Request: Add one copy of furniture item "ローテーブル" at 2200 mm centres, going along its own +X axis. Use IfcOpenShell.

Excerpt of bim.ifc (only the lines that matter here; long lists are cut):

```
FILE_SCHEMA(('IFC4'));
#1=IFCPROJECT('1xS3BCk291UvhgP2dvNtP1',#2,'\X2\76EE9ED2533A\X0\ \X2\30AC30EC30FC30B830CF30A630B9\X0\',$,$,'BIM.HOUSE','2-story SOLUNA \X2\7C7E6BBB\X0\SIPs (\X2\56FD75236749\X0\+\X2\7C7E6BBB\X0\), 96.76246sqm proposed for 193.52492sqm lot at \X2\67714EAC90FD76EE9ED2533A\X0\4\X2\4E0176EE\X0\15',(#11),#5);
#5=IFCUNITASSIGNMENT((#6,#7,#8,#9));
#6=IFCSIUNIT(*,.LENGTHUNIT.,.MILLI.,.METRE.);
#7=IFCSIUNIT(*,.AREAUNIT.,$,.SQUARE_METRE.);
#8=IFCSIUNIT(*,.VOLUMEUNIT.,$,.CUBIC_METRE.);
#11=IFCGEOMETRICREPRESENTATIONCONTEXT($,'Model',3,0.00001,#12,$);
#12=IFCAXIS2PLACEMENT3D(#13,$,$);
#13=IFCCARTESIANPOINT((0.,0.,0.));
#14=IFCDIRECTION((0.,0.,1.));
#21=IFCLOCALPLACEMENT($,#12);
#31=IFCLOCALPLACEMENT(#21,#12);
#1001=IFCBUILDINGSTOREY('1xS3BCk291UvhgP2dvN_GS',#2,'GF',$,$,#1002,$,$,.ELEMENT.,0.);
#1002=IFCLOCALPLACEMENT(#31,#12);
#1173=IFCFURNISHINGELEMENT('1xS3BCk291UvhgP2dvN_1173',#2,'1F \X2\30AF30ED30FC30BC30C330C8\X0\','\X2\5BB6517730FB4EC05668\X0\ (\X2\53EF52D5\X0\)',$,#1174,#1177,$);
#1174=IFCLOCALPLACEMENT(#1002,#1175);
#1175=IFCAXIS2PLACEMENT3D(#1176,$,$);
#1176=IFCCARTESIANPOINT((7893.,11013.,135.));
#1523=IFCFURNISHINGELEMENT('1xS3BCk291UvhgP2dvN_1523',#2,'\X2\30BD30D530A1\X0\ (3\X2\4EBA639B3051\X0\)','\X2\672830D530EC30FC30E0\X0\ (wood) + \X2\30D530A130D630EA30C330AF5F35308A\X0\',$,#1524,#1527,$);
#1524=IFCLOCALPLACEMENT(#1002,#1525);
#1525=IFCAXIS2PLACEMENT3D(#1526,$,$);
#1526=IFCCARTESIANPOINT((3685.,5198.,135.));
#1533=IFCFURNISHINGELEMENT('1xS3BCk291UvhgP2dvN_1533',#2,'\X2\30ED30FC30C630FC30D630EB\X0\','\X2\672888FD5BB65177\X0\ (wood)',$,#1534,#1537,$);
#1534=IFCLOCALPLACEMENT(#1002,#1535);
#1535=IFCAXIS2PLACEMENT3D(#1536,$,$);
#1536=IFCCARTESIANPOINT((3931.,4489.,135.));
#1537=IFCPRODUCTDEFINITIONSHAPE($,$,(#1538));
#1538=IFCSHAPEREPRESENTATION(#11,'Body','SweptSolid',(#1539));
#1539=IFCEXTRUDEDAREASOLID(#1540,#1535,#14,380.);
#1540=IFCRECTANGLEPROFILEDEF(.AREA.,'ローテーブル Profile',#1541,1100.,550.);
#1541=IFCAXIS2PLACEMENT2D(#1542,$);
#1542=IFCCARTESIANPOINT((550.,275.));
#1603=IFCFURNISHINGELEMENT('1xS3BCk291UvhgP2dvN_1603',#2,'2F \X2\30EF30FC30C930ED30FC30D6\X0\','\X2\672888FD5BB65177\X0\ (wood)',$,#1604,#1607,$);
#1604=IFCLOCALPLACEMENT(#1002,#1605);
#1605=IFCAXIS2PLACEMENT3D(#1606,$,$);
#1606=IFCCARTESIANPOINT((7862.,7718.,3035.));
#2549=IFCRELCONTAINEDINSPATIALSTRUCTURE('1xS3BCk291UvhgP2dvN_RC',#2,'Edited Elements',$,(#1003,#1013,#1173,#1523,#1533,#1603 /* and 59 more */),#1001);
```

```python
import ifcopenshell
import ifcopenshell.api.geometry
import ifcopenshell.api.root
import ifcopenshell.util.element
import ifcopenshell.util.placement

model = ifcopenshell.open("bim.ifc")


def reuse_history(source, copy):
    """copy_class also copies each property set's owner history, people and application; keep the originals."""
    for rel in copy.IsDefinedBy:
        if rel.is_a("IfcRelDefinesByProperties") and (history := rel.RelatingPropertyDefinition.OwnerHistory):
            rel.RelatingPropertyDefinition.OwnerHistory = source.OwnerHistory
            ifcopenshell.util.element.remove_deep2(model, history)


source = model.by_guid("1xS3BCk291UvhgP2dvN_1533")
base = ifcopenshell.util.placement.get_local_placement(source.ObjectPlacement)
step = base[:3, 0] * 2200.0

for i in range(1, 2):
    copy = ifcopenshell.api.root.copy_class(model, product=source)
    copy.Representation = ifcopenshell.util.element.copy_deep(
        model, source.Representation, exclude=["IfcGeometricRepresentationContext", "IfcRepresentationMap"]
    )
    reuse_history(source, copy)
    matrix = base.copy()
    matrix[:3, 3] += i * step
    print("added at", matrix[:3, 3].round(3) + 0.0)
    ifcopenshell.api.geometry.edit_object_placement(model, product=copy, matrix=matrix, is_si=False)

model.write("bim_rev.ifc")
```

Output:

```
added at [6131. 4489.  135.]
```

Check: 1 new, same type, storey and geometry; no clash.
